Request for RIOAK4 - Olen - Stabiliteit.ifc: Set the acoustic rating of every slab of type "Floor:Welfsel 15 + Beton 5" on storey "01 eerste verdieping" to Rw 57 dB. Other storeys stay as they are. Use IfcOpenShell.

First a look at what the model holds.

```python
import ifcopenshell
import ifcopenshell.util.element

model = ifcopenshell.open("RIOAK4 - Olen - Stabiliteit.ifc")
print(model.schema)
storey = next(s for s in model.by_type("IfcBuildingStorey") if s.Name == "01 eerste verdieping")
slabs = [e for e in ifcopenshell.util.element.get_decomposition(storey) if e.is_a("IfcSlab")]
seen = {}
for e in slabs:
    element_type = ifcopenshell.util.element.get_type(e)
    key = (element_type.Name if element_type != e and element_type else None, ifcopenshell.util.element.get_pset(e, "Pset_SlabCommon", "AcousticRating"))
    seen[key] = seen.get(key, 0) + 1
for (name, value), count in sorted(seen.items(), key=str):
    print(count, "x", name, "|", value)
```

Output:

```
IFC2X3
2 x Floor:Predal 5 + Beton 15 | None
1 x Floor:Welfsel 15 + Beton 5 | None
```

```python
import ifcopenshell
import ifcopenshell.api.pset
import ifcopenshell.util.element

model = ifcopenshell.open("RIOAK4 - Olen - Stabiliteit.ifc")

storey = next(s for s in model.by_type("IfcBuildingStorey") if s.Name == "01 eerste verdieping")
slabs = [e for e in ifcopenshell.util.element.get_decomposition(storey) if e.is_a("IfcSlab")]

count = 0
for e in slabs:
    element_type = ifcopenshell.util.element.get_type(e)
    if element_type in (None, e) or element_type.Name != "Floor:Welfsel 15 + Beton 5":
        continue
    # add_pset returns the element's existing set when there is one.
    pset = ifcopenshell.api.pset.add_pset(model, product=e, name="Pset_SlabCommon")
    ifcopenshell.api.pset.edit_pset(model, pset=pset, properties={"AcousticRating": "Rw 57 dB"})
    count += 1

print(count, "slabs updated")

model.write("RIOAK4 - Olen - Stabiliteit_v2.ifc")
```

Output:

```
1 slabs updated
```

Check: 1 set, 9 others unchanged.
